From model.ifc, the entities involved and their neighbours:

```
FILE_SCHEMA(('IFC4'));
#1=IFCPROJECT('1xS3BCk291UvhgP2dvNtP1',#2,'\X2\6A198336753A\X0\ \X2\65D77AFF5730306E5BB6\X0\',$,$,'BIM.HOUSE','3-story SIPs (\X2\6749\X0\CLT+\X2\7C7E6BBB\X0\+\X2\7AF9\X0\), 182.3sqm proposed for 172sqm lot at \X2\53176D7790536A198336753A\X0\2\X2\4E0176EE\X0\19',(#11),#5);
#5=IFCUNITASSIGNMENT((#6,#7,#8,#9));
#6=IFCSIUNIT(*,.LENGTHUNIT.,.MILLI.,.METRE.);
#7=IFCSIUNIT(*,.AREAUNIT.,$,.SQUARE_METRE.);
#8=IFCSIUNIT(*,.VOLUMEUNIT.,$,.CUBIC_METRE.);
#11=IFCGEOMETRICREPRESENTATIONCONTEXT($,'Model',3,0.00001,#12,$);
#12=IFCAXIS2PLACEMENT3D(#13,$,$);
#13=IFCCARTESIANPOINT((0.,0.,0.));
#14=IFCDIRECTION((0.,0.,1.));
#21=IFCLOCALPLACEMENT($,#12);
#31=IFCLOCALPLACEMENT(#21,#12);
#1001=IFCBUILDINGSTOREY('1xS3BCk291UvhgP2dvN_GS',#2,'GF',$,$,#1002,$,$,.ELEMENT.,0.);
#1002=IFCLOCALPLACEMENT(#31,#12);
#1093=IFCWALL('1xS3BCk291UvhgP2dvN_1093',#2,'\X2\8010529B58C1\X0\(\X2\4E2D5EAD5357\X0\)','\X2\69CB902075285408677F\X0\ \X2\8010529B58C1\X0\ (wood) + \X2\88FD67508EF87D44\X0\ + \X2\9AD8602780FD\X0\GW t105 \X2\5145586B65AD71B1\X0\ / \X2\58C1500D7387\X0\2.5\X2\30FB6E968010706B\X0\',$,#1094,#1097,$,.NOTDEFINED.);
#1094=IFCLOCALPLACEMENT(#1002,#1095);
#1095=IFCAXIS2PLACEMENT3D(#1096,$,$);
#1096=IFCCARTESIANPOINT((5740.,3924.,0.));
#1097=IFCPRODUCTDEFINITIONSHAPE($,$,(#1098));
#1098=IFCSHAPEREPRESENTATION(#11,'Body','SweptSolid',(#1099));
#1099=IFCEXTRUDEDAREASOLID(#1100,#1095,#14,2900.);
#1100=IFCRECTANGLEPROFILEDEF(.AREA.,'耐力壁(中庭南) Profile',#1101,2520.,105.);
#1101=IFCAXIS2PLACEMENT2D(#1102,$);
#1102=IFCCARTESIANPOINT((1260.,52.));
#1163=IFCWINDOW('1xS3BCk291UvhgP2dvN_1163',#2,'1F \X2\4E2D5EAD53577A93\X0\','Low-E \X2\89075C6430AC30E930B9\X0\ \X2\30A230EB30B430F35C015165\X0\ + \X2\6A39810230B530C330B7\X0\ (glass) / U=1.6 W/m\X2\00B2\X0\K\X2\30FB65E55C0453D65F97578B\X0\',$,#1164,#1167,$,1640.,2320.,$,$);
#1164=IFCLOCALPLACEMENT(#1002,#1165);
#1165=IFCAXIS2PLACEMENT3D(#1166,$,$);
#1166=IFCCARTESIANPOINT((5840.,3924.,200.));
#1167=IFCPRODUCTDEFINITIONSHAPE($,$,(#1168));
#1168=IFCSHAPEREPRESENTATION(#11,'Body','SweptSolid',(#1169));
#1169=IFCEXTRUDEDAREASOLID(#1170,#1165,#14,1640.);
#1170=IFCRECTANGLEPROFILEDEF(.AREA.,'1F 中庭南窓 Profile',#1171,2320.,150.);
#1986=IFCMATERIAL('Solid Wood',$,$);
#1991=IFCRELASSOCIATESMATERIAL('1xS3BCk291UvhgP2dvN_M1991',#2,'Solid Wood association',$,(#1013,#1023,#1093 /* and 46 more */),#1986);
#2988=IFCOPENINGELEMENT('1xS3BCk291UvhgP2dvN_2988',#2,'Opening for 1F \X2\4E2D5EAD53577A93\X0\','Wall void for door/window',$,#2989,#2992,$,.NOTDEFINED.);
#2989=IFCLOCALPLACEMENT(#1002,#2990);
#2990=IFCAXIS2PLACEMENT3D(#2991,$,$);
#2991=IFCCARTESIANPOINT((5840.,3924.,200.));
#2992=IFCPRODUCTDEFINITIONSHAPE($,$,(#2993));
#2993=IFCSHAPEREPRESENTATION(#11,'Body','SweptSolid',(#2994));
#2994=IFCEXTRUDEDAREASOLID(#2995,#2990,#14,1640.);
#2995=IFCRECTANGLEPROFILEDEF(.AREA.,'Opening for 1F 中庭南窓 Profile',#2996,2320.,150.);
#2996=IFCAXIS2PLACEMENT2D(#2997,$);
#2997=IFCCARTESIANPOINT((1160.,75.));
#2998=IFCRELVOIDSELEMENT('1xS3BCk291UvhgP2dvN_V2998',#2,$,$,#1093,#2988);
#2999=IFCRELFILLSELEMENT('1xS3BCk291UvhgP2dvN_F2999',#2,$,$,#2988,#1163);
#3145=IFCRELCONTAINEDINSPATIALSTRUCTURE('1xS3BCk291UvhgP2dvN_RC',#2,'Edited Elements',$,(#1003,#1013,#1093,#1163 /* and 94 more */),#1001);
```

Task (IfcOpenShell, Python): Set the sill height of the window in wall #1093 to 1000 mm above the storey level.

```python
import numpy as np
import ifcopenshell
import ifcopenshell.api.geometry
import ifcopenshell.geom
import ifcopenshell.util.element
import ifcopenshell.util.placement
import ifcopenshell.util.shape
import ifcopenshell.util.unit

model = ifcopenshell.open("model.ifc")
unit_scale = ifcopenshell.util.unit.calculate_unit_scale(model)

window = model.by_guid("1xS3BCk291UvhgP2dvN_1163")
opening = window.FillsVoids[0].RelatingOpeningElement
storey = ifcopenshell.util.element.get_container(window, ifc_class="IfcBuildingStorey")
level = ifcopenshell.util.placement.get_local_placement(storey.ObjectPlacement)[2, 3]

# The opening's origin need not be at the sill, so measure its lowest point.
shape = ifcopenshell.geom.create_shape(ifcopenshell.geom.settings(), opening)
bottom = ifcopenshell.util.shape.get_shape_bottom_elevation(shape, shape.geometry) / unit_scale
dz = level + 1000.0 - bottom

shift = np.array([0.0, 0.0, dz])
# The window is not placed relative to its opening, so move both.
for product in (opening, window):
    matrix = ifcopenshell.util.placement.get_local_placement(product.ObjectPlacement)
    matrix[:3, 3] += shift
    ifcopenshell.api.geometry.edit_object_placement(model, product=product, matrix=matrix, is_si=False)

print(f"moved by {dz * unit_scale:+.3f} m")

model.write("model_v2.ifc")
```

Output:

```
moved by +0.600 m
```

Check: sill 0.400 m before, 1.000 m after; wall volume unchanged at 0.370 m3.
